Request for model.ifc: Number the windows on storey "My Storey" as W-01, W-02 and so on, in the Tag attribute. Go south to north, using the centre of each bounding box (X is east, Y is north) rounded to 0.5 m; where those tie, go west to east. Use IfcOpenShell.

First a look at what the model holds.

```python
import ifcopenshell
import ifcopenshell.util.element
import ifcopenshell.util.placement

model = ifcopenshell.open("model.ifc")
print(model.schema)
storey = next(s for s in model.by_type("IfcBuildingStorey") if s.Name == "My Storey")
windows = [e for e in ifcopenshell.util.element.get_decomposition(storey) if e.is_a("IfcWindow")]
for e in sorted(windows, key=lambda e: e.id()):
    origin = ifcopenshell.util.placement.get_local_placement(e.ObjectPlacement)[:3, 3]
    print(e.id(), e.Tag, e.Name, origin.round(2) + 0.0, sep=" | ")
```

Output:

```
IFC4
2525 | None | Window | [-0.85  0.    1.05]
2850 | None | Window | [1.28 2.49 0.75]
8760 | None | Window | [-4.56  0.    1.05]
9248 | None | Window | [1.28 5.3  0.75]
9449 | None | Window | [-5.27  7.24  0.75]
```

```python
import ifcopenshell
import ifcopenshell.geom
import ifcopenshell.util.element
import ifcopenshell.util.shape

model = ifcopenshell.open("model.ifc")
settings = ifcopenshell.geom.settings()
settings.set("use-world-coords", True)


def centre(element):
    shape = ifcopenshell.geom.create_shape(settings, element)
    return ifcopenshell.util.shape.get_bbox_centroid(shape.geometry)


storey = next(s for s in model.by_type("IfcBuildingStorey") if s.Name == "My Storey")
windows = [e for e in ifcopenshell.util.element.get_decomposition(storey) if e.is_a("IfcWindow")]

# Insertion points can sit at a corner or the storey origin, so sort by the geometry (in metres).
centres = {e: centre(e) for e in windows}
windows.sort(key=lambda e: (round(centres[e][1] / 0.5), centres[e][0]))

for i, e in enumerate(windows, start=1):
    number = f"W-{i:02d}"
    e.Tag = number
    print(e.id(), number)

model.write("model-out.ifc")
```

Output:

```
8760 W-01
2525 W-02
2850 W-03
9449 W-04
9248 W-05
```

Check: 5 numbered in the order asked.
